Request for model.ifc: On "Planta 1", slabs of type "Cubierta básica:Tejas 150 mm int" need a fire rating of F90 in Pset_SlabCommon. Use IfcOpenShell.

First a look at what the model holds.

```python
import ifcopenshell
import ifcopenshell.util.element

model = ifcopenshell.open("model.ifc")
print(model.schema)
storey = next(s for s in model.by_type("IfcBuildingStorey") if s.Name == "Planta 1")
slabs = [e for e in ifcopenshell.util.element.get_decomposition(storey) if e.is_a("IfcSlab")]
seen = {}
for e in slabs:
    element_type = ifcopenshell.util.element.get_type(e)
    key = (element_type.Name if element_type != e and element_type else None, ifcopenshell.util.element.get_pset(e, "Pset_SlabCommon", "FireRating"))
    seen[key] = seen.get(key, 0) + 1
for (name, value), count in sorted(seen.items(), key=str):
    print(count, "x", name, "|", value)
```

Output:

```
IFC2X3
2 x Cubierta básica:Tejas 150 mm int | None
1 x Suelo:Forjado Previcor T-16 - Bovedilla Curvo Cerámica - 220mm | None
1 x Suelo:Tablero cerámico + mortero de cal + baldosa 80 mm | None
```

```python
import ifcopenshell
import ifcopenshell.api.pset
import ifcopenshell.util.element

model = ifcopenshell.open("model.ifc")

storey = next(s for s in model.by_type("IfcBuildingStorey") if s.Name == "Planta 1")
slabs = [e for e in ifcopenshell.util.element.get_decomposition(storey) if e.is_a("IfcSlab")]

count = 0
for e in slabs:
    element_type = ifcopenshell.util.element.get_type(e)
    if element_type in (None, e) or element_type.Name != "Cubierta básica:Tejas 150 mm int":
        continue
    # add_pset returns the element's existing set when there is one.
    pset = ifcopenshell.api.pset.add_pset(model, product=e, name="Pset_SlabCommon")
    ifcopenshell.api.pset.edit_pset(model, pset=pset, properties={"FireRating": "F90"})
    count += 1

print(count, "slabs updated")

model.write("model_rev.ifc")
```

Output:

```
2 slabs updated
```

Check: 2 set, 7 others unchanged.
